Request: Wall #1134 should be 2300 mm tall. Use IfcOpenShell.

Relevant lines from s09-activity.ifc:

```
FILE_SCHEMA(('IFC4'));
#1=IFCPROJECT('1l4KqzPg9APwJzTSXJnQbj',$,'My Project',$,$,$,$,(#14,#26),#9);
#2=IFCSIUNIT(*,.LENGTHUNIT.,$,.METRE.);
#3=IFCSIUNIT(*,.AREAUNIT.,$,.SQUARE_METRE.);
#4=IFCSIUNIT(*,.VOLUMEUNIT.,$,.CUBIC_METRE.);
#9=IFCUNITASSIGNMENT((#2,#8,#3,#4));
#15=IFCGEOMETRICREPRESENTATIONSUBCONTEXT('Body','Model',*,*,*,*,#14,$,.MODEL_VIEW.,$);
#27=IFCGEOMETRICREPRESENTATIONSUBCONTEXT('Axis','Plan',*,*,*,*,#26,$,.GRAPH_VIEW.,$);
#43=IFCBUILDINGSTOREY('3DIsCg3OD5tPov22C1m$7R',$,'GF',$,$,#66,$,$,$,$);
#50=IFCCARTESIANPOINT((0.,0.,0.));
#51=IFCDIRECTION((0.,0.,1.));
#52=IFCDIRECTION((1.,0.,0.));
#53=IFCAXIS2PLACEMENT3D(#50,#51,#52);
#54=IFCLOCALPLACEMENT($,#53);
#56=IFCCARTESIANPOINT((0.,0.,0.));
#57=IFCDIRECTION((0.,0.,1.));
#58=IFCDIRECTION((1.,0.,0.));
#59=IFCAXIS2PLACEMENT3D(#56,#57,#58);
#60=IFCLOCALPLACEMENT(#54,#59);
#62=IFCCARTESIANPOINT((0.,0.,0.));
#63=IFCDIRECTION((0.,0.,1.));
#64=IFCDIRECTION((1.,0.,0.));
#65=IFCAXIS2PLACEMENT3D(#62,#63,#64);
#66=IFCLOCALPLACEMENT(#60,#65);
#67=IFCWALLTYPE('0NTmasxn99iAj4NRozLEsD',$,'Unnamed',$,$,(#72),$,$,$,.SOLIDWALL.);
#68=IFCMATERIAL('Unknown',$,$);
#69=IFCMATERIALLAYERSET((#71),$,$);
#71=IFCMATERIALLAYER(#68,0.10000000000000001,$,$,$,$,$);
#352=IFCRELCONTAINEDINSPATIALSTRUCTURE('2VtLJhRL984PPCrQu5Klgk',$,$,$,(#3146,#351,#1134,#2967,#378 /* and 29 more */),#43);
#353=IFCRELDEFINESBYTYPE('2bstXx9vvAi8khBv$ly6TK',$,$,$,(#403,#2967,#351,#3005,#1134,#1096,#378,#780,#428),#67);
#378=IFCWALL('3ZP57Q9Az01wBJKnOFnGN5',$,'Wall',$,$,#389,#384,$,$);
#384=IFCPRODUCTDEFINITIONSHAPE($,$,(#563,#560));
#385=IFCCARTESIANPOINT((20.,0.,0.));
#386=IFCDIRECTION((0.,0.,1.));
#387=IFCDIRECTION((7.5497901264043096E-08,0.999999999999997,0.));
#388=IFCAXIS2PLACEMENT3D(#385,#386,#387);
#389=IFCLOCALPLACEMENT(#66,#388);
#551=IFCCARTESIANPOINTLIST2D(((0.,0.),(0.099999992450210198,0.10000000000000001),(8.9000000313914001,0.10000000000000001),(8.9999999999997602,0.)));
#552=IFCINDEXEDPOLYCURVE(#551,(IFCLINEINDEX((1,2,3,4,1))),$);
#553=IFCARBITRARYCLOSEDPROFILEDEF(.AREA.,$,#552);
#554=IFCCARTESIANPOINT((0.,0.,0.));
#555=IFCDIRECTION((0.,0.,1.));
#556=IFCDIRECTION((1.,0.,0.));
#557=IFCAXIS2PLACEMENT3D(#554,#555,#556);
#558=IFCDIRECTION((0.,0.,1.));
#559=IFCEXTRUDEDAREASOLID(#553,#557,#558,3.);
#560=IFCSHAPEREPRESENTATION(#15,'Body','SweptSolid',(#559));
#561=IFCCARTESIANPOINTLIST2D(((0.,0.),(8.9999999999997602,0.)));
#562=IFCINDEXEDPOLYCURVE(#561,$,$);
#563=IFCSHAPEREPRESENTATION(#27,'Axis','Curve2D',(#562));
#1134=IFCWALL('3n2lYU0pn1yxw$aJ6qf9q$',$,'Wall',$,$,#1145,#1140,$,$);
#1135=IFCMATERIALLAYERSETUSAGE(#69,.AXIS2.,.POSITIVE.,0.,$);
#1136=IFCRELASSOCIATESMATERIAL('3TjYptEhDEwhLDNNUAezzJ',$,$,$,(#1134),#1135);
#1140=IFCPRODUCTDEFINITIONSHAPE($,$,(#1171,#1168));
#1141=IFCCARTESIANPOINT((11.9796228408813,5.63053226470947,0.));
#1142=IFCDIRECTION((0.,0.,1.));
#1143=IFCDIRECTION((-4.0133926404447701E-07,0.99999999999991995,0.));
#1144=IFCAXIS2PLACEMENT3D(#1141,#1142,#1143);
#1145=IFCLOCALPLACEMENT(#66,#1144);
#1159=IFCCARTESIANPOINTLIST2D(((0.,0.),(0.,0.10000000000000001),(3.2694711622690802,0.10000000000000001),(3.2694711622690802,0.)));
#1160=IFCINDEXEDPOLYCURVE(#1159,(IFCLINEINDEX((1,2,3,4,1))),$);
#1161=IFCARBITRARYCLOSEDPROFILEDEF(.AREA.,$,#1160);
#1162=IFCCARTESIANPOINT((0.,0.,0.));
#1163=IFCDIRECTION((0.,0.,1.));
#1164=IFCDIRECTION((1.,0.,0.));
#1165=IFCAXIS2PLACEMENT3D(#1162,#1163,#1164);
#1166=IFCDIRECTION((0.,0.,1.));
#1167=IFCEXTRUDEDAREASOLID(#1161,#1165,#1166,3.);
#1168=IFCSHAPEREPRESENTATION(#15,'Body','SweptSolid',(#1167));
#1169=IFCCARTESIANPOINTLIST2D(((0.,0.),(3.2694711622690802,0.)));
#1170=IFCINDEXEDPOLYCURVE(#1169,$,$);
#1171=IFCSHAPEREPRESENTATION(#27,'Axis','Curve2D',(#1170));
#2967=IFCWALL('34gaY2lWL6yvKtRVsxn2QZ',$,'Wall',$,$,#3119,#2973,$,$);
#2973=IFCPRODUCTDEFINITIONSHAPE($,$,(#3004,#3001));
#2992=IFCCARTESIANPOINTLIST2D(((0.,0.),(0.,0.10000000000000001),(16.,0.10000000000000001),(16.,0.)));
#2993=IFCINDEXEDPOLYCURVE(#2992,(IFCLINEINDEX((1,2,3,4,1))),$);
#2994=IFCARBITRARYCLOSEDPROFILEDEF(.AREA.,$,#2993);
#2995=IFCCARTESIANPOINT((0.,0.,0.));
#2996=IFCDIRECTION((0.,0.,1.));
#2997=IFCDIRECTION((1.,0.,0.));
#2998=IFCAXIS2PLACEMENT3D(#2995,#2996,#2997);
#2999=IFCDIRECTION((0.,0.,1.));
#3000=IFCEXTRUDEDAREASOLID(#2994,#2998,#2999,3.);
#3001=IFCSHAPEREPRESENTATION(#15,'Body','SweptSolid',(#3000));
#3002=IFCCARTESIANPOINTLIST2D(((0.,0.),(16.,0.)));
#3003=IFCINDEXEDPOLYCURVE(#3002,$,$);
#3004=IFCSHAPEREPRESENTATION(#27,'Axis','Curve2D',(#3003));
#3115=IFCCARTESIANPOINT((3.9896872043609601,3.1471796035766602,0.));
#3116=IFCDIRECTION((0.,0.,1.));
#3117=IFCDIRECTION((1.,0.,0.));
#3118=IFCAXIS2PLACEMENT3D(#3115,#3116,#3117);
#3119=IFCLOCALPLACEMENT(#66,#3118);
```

```python
import ifcopenshell
import ifcopenshell.geom
import ifcopenshell.util.representation
import ifcopenshell.util.shape
import ifcopenshell.util.unit

model = ifcopenshell.open("s09-activity.ifc")
unit_scale = ifcopenshell.util.unit.calculate_unit_scale(model)
settings = ifcopenshell.geom.settings()


def volume(element):
    """Net volume in cubic metres, openings subtracted."""
    shape = ifcopenshell.geom.create_shape(settings, element)
    return ifcopenshell.util.shape.get_volume(shape.geometry)


wall = model.by_id(1134)
before = volume(wall)

body = ifcopenshell.util.representation.get_representation(wall, "Model", "Body")
solid = body.Items[0]
old_height = solid.Depth
solid.Depth = 2.3 / unit_scale
after = volume(wall)

print(f"height {old_height:g} -> {solid.Depth:g}, volume {before:.3f} -> {after:.3f} m3")

model.write("s09-activity-out.ifc")
```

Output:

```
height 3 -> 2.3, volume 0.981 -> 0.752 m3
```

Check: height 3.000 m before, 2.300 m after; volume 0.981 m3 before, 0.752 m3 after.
